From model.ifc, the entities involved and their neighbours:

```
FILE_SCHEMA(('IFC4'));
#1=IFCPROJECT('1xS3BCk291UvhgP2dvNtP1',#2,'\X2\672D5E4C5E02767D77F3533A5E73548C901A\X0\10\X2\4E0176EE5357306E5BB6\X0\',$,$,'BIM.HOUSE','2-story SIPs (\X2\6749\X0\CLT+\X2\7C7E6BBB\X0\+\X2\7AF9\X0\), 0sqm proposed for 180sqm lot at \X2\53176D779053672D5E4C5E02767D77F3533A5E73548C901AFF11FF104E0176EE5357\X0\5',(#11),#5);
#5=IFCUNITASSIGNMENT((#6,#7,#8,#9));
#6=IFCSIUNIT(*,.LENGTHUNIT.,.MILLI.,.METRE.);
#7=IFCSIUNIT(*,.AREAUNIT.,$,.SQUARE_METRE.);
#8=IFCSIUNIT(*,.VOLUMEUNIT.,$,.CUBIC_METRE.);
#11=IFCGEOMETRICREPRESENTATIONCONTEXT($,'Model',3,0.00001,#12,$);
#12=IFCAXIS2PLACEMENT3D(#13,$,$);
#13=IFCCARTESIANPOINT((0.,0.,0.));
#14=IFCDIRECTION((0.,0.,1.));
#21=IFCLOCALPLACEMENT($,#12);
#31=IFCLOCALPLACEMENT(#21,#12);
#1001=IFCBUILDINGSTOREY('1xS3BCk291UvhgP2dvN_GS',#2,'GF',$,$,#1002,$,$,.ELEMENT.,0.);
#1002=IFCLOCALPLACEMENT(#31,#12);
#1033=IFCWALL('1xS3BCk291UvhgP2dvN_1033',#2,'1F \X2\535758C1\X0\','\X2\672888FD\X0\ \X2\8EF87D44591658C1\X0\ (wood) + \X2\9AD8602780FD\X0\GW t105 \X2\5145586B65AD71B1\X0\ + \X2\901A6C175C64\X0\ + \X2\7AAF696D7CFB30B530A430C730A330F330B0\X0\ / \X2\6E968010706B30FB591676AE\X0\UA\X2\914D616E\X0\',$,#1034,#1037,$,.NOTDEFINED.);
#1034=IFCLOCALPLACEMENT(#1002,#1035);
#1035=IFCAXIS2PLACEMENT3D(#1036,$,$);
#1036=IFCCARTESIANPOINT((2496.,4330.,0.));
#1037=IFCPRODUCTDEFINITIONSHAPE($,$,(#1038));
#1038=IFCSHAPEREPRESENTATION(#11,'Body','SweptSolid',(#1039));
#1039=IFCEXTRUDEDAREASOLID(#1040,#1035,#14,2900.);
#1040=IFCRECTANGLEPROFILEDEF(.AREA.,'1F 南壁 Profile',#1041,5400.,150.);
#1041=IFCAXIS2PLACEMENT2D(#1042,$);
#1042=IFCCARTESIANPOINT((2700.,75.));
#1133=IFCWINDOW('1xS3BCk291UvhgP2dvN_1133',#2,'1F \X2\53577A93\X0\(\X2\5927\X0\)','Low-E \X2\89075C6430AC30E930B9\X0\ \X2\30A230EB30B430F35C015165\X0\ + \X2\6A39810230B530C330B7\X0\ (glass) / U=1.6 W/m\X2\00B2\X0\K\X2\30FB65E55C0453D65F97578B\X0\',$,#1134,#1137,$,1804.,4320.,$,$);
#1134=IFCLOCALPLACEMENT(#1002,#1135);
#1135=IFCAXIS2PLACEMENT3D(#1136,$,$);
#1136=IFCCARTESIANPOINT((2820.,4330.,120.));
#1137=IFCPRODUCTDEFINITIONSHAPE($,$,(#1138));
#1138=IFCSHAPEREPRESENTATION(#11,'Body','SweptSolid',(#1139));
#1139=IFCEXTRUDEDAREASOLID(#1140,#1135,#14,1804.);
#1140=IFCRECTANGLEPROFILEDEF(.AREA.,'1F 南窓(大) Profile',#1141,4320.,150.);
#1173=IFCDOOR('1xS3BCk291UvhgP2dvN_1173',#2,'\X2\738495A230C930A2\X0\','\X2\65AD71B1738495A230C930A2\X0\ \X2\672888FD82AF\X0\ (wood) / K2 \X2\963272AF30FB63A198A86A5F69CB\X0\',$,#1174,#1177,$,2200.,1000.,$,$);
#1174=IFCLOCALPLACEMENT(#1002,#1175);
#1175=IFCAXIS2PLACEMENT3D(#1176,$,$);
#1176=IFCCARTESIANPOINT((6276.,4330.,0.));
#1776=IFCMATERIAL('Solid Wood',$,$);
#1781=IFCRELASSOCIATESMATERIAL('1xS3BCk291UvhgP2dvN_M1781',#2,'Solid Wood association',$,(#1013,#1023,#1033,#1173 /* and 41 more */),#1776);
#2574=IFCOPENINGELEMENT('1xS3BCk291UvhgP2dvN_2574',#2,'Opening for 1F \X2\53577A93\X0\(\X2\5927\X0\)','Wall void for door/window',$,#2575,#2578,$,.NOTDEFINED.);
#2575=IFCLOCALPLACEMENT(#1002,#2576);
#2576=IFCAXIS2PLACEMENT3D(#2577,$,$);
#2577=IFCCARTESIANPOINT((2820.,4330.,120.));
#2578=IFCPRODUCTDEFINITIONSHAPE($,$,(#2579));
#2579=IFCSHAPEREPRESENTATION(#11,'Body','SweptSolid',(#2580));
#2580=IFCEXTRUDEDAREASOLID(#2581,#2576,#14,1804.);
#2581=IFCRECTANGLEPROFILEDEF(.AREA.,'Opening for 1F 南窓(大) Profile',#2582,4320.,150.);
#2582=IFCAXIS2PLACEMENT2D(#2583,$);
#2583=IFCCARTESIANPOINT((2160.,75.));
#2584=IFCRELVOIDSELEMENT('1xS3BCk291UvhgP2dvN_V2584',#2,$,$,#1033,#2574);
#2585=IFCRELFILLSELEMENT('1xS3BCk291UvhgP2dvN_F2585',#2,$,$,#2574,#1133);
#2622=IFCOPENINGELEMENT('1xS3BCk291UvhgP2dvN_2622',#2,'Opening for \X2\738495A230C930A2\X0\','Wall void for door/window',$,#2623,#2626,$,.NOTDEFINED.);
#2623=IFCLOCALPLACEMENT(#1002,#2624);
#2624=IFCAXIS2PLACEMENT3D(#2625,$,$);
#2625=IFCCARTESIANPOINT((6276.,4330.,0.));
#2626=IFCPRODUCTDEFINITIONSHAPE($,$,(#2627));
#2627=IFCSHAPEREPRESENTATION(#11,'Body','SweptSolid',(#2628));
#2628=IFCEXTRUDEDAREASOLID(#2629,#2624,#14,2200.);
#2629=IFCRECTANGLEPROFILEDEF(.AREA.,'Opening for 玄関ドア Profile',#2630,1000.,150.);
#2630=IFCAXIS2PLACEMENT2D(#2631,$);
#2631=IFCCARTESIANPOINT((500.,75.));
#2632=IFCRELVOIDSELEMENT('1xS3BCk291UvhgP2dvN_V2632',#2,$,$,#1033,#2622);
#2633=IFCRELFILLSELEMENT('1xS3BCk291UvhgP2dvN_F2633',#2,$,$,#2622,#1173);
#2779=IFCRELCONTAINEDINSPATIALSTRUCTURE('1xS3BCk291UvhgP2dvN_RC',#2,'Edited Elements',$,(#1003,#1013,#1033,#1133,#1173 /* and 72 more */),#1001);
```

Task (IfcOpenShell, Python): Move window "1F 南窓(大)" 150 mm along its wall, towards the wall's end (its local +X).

```python
import ifcopenshell
import ifcopenshell.api.geometry
import ifcopenshell.util.placement
import ifcopenshell.util.unit

model = ifcopenshell.open("model.ifc")
unit_scale = ifcopenshell.util.unit.calculate_unit_scale(model)

window = model.by_guid("1xS3BCk291UvhgP2dvN_1133")
opening = window.FillsVoids[0].RelatingOpeningElement
wall = opening.VoidsElements[0].RelatingBuildingElement

wall_matrix = ifcopenshell.util.placement.get_local_placement(wall.ObjectPlacement)
shift = wall_matrix[:3, 0] * 0.15 / unit_scale
before = ifcopenshell.util.placement.get_local_placement(window.ObjectPlacement)[:3, 3].copy()

# The window is not placed relative to its opening, so move both.
for product in (opening, window):
    matrix = ifcopenshell.util.placement.get_local_placement(product.ObjectPlacement)
    matrix[:3, 3] += shift
    ifcopenshell.api.geometry.edit_object_placement(model, product=product, matrix=matrix, is_si=False)

after = ifcopenshell.util.placement.get_local_placement(window.ObjectPlacement)[:3, 3]
print("window moved by", (after - before).round(3) + 0.0)

model.write("model-out.ifc")
```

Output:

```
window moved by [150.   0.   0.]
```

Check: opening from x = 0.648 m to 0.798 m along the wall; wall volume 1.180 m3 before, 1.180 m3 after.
